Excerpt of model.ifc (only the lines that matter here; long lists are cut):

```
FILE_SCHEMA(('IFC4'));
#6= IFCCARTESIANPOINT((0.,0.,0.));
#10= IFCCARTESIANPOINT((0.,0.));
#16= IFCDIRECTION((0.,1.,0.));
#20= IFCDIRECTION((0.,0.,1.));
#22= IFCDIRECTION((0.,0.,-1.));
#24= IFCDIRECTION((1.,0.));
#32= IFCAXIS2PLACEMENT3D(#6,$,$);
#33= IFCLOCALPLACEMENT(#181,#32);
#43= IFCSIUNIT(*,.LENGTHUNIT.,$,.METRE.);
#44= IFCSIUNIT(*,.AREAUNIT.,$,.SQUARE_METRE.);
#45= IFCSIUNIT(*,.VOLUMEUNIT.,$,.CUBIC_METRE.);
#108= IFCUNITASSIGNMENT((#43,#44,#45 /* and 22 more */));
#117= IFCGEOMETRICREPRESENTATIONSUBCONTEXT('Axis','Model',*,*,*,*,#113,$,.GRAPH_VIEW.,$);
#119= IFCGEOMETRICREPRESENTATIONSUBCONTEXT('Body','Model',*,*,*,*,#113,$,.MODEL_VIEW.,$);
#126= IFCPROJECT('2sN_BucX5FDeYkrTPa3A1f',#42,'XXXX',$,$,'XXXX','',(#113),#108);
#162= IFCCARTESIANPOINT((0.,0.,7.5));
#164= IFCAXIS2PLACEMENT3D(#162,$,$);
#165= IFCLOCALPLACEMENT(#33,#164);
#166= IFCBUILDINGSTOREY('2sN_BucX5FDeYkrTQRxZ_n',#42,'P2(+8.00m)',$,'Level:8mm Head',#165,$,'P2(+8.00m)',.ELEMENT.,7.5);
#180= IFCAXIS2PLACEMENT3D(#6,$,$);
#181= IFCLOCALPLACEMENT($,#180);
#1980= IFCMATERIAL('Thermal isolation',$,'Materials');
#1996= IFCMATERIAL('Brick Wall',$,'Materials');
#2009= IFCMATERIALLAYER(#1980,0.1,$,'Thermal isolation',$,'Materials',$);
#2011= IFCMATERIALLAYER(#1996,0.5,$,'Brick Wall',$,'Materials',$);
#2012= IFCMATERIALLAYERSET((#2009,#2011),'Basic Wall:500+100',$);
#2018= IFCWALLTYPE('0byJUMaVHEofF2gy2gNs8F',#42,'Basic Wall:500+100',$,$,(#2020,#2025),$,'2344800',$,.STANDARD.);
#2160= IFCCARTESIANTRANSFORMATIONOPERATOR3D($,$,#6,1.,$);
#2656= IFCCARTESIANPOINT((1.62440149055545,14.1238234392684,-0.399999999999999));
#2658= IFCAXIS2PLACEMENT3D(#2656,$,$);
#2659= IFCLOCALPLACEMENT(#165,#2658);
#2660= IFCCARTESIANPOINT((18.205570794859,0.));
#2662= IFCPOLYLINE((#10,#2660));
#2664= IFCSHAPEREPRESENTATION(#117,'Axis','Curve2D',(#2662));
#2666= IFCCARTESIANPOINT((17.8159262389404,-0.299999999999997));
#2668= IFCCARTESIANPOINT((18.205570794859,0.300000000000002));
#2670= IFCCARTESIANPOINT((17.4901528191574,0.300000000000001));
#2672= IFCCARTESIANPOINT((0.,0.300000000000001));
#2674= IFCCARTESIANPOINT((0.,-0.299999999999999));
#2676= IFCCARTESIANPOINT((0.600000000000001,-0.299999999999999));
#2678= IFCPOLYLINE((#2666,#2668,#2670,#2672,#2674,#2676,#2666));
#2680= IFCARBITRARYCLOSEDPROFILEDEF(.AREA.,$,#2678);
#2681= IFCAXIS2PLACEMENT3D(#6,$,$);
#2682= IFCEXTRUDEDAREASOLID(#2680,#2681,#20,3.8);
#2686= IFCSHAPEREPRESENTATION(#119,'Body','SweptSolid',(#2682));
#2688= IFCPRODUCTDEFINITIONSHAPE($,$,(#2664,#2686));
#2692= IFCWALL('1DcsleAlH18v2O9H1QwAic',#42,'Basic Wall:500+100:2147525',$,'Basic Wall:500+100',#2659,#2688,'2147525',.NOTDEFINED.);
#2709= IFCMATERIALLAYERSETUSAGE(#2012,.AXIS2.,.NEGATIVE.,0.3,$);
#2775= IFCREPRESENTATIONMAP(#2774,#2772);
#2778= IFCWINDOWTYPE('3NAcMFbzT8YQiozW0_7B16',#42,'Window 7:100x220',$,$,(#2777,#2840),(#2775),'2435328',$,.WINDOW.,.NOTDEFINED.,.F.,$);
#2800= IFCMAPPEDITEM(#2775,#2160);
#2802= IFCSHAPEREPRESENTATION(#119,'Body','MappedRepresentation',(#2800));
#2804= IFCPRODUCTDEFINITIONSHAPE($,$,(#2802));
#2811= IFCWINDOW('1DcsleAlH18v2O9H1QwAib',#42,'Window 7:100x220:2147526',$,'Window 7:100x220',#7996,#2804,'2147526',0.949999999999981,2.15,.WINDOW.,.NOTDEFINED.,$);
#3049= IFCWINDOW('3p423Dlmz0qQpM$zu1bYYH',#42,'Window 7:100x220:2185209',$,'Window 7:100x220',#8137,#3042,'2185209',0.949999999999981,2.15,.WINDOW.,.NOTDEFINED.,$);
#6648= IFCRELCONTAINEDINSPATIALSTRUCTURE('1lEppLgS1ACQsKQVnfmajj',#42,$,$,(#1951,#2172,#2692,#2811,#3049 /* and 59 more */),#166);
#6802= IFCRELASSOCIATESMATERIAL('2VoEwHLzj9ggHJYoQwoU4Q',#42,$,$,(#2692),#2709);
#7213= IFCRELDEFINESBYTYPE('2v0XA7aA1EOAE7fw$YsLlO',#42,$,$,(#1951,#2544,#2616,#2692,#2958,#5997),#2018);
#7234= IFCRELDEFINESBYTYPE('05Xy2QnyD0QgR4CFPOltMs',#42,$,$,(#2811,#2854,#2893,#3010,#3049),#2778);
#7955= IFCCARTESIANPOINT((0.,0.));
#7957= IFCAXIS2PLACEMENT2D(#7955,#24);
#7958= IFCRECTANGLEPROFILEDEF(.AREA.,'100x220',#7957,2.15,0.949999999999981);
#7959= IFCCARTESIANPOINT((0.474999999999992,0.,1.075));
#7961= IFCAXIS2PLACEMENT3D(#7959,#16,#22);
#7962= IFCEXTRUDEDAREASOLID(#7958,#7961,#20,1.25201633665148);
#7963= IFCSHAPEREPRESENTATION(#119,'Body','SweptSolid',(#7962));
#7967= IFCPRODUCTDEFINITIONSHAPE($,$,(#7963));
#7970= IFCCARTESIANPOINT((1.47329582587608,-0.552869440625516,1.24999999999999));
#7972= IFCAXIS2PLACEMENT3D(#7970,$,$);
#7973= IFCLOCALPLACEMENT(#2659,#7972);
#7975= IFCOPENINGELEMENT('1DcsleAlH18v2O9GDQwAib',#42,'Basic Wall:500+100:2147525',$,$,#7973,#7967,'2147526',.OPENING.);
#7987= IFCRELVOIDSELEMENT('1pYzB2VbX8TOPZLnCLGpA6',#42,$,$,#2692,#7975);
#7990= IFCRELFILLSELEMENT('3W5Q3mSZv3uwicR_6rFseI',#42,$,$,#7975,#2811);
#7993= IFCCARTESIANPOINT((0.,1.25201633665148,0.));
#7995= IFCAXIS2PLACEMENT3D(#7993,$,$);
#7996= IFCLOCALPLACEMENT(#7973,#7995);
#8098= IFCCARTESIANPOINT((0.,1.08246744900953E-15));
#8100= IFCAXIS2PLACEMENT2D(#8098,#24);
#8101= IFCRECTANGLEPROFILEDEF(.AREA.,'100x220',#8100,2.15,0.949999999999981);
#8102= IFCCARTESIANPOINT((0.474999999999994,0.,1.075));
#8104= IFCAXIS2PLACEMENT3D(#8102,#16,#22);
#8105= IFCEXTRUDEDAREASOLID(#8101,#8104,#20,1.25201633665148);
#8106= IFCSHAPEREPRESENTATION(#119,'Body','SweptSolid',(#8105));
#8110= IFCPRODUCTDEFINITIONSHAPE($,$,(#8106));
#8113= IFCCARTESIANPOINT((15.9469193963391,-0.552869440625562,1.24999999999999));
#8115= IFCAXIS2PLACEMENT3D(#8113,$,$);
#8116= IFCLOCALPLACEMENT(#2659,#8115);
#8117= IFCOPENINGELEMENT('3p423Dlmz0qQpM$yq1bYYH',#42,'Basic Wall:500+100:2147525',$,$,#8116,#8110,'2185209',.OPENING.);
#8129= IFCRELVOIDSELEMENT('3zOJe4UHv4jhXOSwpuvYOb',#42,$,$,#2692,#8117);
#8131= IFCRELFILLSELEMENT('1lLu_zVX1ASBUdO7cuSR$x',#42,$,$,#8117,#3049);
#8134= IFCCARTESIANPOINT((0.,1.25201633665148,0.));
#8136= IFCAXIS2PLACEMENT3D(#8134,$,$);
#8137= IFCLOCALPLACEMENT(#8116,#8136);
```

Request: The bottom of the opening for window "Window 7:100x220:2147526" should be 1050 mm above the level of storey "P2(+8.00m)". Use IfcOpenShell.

```python
import numpy as np
import ifcopenshell
import ifcopenshell.api.geometry
import ifcopenshell.geom
import ifcopenshell.util.element
import ifcopenshell.util.placement
import ifcopenshell.util.shape
import ifcopenshell.util.unit

model = ifcopenshell.open("model.ifc")
unit_scale = ifcopenshell.util.unit.calculate_unit_scale(model)

window = model.by_guid("1DcsleAlH18v2O9H1QwAib")
opening = window.FillsVoids[0].RelatingOpeningElement
storey = ifcopenshell.util.element.get_container(window, ifc_class="IfcBuildingStorey")
level = ifcopenshell.util.placement.get_local_placement(storey.ObjectPlacement)[2, 3]

# The opening's origin need not be at the sill, so measure its lowest point.
shape = ifcopenshell.geom.create_shape(ifcopenshell.geom.settings(), opening)
bottom = ifcopenshell.util.shape.get_shape_bottom_elevation(shape, shape.geometry) / unit_scale
dz = level + 1.05 / unit_scale - bottom

shift = np.array([0.0, 0.0, dz])
# The window is placed relative to its opening, so it follows when the opening moves.
matrix = ifcopenshell.util.placement.get_local_placement(opening.ObjectPlacement)
matrix[:3, 3] += shift
ifcopenshell.api.geometry.edit_object_placement(
    model, product=opening, matrix=matrix, is_si=False, should_transform_children=True
)

print(f"moved by {dz * unit_scale:+.3f} m")

model.write("model_rev.ifc")
```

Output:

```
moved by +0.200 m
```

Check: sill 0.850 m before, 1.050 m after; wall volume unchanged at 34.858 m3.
